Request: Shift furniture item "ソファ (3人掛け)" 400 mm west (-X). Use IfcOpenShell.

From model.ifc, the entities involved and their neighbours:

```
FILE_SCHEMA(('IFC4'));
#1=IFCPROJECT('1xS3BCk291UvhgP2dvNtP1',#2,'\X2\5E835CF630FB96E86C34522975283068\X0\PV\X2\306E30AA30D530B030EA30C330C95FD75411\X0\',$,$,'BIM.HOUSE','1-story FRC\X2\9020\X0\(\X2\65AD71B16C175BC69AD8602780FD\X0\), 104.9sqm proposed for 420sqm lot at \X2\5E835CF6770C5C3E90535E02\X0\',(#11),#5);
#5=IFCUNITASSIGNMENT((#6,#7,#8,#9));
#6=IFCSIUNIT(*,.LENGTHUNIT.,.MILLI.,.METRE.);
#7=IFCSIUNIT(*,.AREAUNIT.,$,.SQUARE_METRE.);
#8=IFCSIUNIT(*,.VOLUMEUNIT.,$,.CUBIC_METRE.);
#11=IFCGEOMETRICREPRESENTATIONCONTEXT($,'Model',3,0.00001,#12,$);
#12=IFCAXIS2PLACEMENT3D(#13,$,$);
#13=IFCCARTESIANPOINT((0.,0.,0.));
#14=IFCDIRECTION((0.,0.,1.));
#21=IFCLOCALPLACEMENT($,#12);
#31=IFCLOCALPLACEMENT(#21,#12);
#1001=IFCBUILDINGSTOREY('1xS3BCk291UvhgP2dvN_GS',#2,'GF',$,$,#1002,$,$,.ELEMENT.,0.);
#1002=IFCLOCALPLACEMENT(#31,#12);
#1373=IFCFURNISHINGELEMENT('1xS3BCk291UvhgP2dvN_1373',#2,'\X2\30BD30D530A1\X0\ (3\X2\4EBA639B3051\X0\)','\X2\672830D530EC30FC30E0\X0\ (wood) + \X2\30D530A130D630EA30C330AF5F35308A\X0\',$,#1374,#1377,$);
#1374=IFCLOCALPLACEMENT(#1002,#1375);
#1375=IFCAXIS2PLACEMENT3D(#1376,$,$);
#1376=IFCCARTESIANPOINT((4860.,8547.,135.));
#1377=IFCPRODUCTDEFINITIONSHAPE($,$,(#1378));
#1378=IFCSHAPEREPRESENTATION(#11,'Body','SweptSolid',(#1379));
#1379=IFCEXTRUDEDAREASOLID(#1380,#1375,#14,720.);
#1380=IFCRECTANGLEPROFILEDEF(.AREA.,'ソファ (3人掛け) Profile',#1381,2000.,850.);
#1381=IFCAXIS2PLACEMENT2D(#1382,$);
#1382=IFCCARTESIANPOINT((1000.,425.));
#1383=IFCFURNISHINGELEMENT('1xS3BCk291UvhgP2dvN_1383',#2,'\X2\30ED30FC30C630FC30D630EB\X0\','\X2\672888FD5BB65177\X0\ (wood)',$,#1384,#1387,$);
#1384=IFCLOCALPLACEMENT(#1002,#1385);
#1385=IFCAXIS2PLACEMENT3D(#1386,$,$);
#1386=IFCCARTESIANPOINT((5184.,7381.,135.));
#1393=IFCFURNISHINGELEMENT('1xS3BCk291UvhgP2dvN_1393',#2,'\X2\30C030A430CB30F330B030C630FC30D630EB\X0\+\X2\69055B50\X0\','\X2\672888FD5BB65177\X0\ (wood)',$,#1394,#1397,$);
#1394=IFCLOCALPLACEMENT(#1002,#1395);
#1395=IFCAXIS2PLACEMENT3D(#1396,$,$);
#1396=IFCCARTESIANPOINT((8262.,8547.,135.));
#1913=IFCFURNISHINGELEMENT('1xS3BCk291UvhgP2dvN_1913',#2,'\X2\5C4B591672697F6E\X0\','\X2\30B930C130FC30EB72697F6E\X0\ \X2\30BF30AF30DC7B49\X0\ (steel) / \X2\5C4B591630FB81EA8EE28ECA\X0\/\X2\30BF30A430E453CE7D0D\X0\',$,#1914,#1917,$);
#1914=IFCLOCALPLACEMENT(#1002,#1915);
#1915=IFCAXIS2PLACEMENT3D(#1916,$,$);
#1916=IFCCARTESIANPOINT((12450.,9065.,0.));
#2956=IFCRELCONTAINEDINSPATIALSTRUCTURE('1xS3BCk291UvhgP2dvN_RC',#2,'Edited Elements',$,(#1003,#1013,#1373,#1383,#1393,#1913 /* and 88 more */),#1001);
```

```python
import ifcopenshell
import ifcopenshell.api.geometry
import ifcopenshell.util.placement
import ifcopenshell.util.unit

model = ifcopenshell.open("model.ifc")
unit_scale = ifcopenshell.util.unit.calculate_unit_scale(model)

item = model.by_id(1373)
matrix = ifcopenshell.util.placement.get_local_placement(item.ObjectPlacement)
matrix[0, 3] -= 0.4 / unit_scale
ifcopenshell.api.geometry.edit_object_placement(model, product=item, matrix=matrix, is_si=False)

print(ifcopenshell.util.placement.get_local_placement(item.ObjectPlacement).round(3) + 0.0)

model.write("model_edited.ifc")
```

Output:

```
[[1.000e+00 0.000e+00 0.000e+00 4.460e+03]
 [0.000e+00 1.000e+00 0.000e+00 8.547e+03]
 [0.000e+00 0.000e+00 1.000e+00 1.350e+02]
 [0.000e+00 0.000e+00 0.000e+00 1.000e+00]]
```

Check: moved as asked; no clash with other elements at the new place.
